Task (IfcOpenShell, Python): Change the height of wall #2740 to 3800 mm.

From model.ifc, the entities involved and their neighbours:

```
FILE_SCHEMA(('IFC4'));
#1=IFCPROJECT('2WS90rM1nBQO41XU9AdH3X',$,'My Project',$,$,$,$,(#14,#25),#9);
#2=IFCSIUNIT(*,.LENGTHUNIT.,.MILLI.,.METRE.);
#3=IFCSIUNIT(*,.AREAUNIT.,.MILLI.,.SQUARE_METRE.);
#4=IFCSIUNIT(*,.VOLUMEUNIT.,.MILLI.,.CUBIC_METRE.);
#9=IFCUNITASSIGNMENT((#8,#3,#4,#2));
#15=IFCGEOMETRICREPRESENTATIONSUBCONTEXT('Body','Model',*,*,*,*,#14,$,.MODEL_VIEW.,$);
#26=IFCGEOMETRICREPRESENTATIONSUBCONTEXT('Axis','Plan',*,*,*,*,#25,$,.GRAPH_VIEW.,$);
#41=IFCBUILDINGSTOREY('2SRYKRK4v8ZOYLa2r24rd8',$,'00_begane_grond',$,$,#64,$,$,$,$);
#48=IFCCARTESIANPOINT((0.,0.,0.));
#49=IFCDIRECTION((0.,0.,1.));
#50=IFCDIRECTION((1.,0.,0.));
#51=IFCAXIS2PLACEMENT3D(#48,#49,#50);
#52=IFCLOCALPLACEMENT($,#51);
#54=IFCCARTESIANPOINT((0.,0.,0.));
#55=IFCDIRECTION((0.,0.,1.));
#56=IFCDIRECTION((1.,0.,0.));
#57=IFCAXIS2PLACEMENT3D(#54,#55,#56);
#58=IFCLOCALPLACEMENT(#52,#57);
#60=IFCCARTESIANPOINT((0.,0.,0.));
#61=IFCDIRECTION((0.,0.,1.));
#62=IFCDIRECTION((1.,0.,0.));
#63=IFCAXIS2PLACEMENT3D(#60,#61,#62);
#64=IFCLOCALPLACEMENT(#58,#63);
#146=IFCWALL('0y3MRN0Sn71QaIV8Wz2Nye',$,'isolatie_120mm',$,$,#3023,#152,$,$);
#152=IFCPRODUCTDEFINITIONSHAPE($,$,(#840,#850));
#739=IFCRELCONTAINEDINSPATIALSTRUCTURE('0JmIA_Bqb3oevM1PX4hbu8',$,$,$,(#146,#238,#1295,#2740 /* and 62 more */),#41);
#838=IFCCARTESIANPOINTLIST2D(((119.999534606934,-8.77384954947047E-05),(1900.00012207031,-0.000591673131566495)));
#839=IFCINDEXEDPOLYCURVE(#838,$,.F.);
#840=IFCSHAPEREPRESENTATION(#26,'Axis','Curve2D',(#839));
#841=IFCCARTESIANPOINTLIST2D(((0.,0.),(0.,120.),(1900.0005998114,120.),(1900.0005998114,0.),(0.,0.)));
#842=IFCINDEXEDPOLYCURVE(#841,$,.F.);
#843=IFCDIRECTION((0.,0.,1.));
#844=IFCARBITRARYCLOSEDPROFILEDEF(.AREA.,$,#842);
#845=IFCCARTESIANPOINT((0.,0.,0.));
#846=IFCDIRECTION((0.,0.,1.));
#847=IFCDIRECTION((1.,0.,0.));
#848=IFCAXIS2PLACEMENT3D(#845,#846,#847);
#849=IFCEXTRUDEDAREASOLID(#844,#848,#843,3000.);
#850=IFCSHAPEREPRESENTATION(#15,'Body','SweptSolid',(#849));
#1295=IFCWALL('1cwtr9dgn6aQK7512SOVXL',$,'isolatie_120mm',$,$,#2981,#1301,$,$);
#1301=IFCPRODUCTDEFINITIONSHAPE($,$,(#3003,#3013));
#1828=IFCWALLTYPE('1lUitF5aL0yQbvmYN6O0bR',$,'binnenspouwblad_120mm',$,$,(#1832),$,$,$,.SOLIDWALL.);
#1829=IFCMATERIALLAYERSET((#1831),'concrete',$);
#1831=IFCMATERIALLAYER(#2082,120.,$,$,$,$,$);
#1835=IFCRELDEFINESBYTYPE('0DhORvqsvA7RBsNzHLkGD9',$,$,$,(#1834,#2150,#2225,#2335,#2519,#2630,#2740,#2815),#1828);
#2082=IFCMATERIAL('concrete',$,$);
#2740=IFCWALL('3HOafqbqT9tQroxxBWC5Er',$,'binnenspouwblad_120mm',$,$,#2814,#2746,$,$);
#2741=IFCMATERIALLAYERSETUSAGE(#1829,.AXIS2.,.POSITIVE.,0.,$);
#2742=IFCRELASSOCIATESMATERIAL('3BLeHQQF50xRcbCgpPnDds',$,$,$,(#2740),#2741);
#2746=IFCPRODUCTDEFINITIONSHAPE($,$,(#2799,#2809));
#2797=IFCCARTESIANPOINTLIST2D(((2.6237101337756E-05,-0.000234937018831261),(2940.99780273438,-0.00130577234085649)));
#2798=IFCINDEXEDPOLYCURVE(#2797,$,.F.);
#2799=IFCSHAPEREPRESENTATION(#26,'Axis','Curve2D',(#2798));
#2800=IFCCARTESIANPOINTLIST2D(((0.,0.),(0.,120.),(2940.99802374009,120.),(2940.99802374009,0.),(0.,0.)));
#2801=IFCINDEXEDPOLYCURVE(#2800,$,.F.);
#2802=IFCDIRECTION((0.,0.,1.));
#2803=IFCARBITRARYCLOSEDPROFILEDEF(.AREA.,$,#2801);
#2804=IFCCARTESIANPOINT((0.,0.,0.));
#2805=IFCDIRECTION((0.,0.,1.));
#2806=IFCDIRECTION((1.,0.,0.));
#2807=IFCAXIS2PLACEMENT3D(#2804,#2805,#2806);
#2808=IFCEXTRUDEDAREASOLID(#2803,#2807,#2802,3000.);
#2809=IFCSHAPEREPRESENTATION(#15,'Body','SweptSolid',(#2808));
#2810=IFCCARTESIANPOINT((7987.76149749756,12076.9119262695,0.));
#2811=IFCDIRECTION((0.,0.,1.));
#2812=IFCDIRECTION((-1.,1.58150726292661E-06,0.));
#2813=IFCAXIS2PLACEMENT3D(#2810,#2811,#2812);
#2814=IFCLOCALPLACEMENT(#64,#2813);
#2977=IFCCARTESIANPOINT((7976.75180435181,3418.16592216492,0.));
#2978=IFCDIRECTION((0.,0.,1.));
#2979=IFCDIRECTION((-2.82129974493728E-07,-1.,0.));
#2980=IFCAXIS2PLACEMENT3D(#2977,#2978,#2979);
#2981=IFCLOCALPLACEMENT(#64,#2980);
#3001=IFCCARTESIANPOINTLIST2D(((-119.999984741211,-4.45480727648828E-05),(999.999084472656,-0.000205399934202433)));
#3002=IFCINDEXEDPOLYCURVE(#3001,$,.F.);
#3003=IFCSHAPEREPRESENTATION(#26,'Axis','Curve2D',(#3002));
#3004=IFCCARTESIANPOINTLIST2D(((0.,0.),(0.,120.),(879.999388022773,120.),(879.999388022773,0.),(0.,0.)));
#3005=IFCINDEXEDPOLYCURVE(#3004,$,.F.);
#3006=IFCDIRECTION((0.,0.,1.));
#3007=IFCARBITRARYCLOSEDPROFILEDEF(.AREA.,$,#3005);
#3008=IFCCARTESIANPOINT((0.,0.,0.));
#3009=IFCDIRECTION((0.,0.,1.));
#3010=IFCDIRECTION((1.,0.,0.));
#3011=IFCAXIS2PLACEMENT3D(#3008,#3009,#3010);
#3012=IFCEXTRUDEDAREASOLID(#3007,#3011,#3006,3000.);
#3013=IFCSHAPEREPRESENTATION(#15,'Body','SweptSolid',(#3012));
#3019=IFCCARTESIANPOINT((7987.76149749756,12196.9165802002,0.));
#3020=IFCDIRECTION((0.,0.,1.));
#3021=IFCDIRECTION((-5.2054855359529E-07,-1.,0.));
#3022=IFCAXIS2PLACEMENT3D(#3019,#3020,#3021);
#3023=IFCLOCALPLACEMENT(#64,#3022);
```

```python
import ifcopenshell
import ifcopenshell.geom
import ifcopenshell.util.representation
import ifcopenshell.util.shape
import ifcopenshell.util.unit

model = ifcopenshell.open("model.ifc")
unit_scale = ifcopenshell.util.unit.calculate_unit_scale(model)
settings = ifcopenshell.geom.settings()


def volume(element):
    """Net volume in cubic metres, openings subtracted."""
    shape = ifcopenshell.geom.create_shape(settings, element)
    return ifcopenshell.util.shape.get_volume(shape.geometry)


wall = model.by_guid("3HOafqbqT9tQroxxBWC5Er")
before = volume(wall)

body = ifcopenshell.util.representation.get_representation(wall, "Model", "Body")
solid = body.Items[0]
old_height = solid.Depth
solid.Depth = 3.8 / unit_scale
after = volume(wall)

print(f"height {old_height:g} -> {solid.Depth:g}, volume {before:.3f} -> {after:.3f} m3")

model.write("model_updated.ifc")
```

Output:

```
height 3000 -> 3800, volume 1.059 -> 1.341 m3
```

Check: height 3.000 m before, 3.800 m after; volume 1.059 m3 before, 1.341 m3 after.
